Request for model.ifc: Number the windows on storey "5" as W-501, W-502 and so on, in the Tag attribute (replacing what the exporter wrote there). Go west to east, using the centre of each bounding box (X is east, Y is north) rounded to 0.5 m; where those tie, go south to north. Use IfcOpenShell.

First a look at what the model holds.

```python
import ifcopenshell
import ifcopenshell.util.element
import ifcopenshell.util.placement

model = ifcopenshell.open("model.ifc")
print(model.schema)
storey = next(s for s in model.by_type("IfcBuildingStorey") if s.Name == "5")
windows = [e for e in ifcopenshell.util.element.get_decomposition(storey) if e.is_a("IfcWindow")]
for e in sorted(windows, key=lambda e: e.id()):
    origin = ifcopenshell.util.placement.get_local_placement(e.ObjectPlacement)[:3, 3]
    print(e.id(), e.Tag, e.Name, origin.round(2) + 0.0, sep=" | ")
```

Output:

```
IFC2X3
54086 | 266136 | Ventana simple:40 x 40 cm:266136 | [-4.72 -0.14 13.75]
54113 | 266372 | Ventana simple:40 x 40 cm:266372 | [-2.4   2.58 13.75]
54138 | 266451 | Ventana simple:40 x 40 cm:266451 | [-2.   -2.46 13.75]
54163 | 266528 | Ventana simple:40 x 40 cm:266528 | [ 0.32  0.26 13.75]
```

```python
import ifcopenshell
import ifcopenshell.geom
import ifcopenshell.util.element
import ifcopenshell.util.shape

model = ifcopenshell.open("model.ifc")
settings = ifcopenshell.geom.settings()
settings.set("use-world-coords", True)


def centre(element):
    shape = ifcopenshell.geom.create_shape(settings, element)
    return ifcopenshell.util.shape.get_bbox_centroid(shape.geometry)


storey = next(s for s in model.by_type("IfcBuildingStorey") if s.Name == "5")
windows = [e for e in ifcopenshell.util.element.get_decomposition(storey) if e.is_a("IfcWindow")]

# Insertion points can sit at a corner or the storey origin, so sort by the geometry (in metres).
centres = {e: centre(e) for e in windows}
windows.sort(key=lambda e: (round(centres[e][0] / 0.5), centres[e][1]))

for i, e in enumerate(windows, start=1):
    number = f"W-5{i:02d}"
    e.Tag = number
    print(e.id(), number)

model.write("model-out.ifc")
```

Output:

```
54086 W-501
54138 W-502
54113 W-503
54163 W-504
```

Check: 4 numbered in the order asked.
